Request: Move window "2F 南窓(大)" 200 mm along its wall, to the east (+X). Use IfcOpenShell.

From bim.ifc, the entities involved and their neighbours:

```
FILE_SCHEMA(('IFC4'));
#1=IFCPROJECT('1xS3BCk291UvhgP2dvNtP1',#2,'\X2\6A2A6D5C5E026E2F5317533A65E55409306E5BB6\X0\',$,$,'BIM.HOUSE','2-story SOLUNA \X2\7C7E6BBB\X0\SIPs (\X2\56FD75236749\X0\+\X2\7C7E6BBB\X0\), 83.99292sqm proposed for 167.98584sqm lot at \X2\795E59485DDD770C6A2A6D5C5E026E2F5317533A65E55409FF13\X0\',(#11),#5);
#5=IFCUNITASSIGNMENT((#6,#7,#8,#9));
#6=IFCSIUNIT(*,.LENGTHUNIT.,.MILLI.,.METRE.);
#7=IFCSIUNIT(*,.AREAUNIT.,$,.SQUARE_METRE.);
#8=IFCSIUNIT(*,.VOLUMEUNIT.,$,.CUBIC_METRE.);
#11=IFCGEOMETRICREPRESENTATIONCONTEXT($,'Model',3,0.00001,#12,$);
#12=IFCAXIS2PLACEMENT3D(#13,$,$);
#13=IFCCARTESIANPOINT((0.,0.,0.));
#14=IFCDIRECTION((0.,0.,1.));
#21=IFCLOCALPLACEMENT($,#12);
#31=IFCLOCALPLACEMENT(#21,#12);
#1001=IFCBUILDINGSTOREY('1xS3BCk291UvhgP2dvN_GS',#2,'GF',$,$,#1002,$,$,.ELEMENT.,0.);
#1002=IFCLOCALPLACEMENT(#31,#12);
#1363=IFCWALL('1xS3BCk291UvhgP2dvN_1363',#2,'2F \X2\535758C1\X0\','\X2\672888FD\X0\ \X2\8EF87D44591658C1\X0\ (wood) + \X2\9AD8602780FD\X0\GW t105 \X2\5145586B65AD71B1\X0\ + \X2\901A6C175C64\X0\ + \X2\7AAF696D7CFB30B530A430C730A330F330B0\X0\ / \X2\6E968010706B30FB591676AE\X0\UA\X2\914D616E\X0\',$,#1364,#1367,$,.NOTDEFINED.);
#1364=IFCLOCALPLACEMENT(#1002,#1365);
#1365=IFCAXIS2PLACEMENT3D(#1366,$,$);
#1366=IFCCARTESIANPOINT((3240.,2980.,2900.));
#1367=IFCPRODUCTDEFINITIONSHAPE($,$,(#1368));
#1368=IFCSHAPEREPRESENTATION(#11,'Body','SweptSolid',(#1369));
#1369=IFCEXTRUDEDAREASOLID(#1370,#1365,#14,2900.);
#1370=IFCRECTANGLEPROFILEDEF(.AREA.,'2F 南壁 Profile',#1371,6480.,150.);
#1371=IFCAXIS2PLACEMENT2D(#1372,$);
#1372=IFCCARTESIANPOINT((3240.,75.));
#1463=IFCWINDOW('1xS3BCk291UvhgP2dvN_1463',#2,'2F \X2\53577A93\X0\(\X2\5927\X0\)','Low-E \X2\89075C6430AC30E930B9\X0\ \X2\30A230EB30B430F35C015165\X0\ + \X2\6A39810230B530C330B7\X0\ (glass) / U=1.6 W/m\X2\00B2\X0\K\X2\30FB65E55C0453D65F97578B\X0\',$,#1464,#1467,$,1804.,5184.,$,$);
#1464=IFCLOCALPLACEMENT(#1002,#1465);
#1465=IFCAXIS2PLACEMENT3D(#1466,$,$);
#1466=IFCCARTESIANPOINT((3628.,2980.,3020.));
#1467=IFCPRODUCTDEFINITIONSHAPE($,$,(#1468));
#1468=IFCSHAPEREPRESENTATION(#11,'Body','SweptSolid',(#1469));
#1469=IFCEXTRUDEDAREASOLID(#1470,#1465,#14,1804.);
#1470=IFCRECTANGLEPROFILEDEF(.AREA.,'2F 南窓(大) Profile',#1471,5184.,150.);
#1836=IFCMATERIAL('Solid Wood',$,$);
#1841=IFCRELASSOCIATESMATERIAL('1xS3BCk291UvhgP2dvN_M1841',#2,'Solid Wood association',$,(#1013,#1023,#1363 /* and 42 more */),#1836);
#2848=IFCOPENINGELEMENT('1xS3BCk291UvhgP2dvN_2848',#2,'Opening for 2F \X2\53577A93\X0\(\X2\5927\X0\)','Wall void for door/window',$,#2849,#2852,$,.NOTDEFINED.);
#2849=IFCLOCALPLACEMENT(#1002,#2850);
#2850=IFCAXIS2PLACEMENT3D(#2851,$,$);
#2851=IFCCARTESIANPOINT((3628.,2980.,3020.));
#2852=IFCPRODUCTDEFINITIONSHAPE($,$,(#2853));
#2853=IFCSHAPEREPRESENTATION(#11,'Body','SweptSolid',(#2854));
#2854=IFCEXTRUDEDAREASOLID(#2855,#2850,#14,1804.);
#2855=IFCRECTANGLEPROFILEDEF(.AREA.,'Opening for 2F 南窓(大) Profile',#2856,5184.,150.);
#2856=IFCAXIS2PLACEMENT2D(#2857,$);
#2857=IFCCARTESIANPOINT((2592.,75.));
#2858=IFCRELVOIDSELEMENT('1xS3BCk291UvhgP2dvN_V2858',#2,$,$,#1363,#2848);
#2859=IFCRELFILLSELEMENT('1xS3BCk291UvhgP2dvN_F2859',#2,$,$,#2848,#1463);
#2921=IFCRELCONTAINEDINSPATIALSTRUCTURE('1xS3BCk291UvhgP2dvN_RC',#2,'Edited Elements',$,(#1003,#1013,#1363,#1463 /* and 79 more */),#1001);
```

```python
import ifcopenshell
import ifcopenshell.api.geometry
import ifcopenshell.util.placement
import ifcopenshell.util.unit

model = ifcopenshell.open("bim.ifc")
unit_scale = ifcopenshell.util.unit.calculate_unit_scale(model)

window = model.by_guid("1xS3BCk291UvhgP2dvN_1463")
opening = window.FillsVoids[0].RelatingOpeningElement
wall = opening.VoidsElements[0].RelatingBuildingElement

wall_matrix = ifcopenshell.util.placement.get_local_placement(wall.ObjectPlacement)
shift = wall_matrix[:3, 0] * 0.2 / unit_scale
before = ifcopenshell.util.placement.get_local_placement(window.ObjectPlacement)[:3, 3].copy()

# The window is not placed relative to its opening, so move both.
for product in (opening, window):
    matrix = ifcopenshell.util.placement.get_local_placement(product.ObjectPlacement)
    matrix[:3, 3] += shift
    ifcopenshell.api.geometry.edit_object_placement(model, product=product, matrix=matrix, is_si=False)

after = ifcopenshell.util.placement.get_local_placement(window.ObjectPlacement)[:3, 3]
print("window moved by", (after - before).round(3) + 0.0)

model.write("bim-out.ifc")
```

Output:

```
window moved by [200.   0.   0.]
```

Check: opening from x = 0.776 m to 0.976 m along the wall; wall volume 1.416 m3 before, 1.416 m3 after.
